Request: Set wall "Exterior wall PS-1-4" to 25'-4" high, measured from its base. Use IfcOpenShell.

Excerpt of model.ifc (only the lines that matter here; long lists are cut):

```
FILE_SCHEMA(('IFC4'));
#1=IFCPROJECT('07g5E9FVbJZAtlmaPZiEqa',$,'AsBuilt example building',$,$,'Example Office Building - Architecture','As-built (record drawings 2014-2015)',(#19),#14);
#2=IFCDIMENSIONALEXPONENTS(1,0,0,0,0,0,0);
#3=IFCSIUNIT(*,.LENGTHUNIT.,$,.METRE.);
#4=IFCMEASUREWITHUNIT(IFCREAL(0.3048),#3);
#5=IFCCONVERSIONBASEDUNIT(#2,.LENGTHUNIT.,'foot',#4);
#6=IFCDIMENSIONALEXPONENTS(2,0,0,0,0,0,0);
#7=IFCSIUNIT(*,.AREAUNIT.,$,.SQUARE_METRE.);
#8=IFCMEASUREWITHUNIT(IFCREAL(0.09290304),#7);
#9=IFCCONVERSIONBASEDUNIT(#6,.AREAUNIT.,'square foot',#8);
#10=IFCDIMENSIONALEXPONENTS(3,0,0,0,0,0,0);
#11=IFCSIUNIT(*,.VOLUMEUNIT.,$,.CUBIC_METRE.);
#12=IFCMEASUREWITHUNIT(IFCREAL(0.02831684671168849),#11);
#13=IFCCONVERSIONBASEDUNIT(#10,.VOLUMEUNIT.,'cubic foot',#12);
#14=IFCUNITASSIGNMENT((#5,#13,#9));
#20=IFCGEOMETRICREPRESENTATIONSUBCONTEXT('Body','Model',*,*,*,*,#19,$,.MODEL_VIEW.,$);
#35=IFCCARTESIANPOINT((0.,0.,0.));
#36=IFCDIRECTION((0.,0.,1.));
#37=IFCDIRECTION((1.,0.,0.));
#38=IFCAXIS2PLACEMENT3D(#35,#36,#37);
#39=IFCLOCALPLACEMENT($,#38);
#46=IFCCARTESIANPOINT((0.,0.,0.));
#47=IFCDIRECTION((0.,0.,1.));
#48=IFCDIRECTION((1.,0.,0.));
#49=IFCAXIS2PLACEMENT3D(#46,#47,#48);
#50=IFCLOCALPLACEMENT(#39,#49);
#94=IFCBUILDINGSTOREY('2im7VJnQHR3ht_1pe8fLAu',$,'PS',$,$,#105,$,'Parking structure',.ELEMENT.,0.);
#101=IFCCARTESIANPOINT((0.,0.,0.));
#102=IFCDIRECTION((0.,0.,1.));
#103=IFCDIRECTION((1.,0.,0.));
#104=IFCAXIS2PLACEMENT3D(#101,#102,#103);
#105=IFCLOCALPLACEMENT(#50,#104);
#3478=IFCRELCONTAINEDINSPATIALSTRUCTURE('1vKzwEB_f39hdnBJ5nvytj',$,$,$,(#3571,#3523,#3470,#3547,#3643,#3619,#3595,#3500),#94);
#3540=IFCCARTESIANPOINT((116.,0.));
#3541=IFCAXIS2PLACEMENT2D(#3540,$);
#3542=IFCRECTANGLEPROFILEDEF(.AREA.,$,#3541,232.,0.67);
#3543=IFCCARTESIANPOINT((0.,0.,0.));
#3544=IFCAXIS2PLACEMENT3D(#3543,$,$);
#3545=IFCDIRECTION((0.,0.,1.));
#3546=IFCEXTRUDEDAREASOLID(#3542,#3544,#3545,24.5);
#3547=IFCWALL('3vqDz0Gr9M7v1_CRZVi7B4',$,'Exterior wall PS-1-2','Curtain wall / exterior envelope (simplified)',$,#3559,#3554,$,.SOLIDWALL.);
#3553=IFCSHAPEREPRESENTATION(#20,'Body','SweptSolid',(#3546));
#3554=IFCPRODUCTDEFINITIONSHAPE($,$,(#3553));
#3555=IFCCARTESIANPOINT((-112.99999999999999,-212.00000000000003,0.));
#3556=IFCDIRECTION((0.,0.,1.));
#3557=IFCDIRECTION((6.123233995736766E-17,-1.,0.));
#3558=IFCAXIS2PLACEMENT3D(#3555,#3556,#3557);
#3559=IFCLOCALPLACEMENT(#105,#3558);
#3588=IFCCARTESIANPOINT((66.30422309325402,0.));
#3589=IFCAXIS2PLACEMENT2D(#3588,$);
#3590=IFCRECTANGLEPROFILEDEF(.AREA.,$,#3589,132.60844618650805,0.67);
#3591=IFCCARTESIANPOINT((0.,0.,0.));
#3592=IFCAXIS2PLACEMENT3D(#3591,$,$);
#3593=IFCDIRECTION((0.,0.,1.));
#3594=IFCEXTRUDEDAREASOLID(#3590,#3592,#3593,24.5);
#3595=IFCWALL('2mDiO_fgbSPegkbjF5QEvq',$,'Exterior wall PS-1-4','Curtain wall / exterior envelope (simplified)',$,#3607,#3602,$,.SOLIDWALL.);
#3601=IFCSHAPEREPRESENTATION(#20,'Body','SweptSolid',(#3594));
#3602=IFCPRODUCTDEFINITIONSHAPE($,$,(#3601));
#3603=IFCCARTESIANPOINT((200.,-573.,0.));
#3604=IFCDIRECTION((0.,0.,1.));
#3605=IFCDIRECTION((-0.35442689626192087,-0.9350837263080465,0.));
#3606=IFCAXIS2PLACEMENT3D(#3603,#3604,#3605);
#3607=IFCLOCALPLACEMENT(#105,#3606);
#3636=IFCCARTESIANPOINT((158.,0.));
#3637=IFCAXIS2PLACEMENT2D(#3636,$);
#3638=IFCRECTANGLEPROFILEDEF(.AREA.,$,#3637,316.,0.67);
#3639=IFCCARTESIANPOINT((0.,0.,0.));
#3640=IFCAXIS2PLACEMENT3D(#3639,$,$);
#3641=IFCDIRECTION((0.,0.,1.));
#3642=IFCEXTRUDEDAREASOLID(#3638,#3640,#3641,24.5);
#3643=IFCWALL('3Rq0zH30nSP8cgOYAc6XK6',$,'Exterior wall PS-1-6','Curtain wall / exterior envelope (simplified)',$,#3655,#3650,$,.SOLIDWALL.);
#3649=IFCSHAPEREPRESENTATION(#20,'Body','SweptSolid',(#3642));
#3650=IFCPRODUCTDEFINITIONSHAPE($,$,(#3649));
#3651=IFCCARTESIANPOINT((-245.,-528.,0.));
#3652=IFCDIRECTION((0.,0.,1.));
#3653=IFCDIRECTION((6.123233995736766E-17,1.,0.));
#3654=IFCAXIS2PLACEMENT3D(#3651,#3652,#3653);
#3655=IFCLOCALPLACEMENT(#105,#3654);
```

```python
import ifcopenshell
import ifcopenshell.geom
import ifcopenshell.util.representation
import ifcopenshell.util.shape
import ifcopenshell.util.unit

model = ifcopenshell.open("model.ifc")
unit_scale = ifcopenshell.util.unit.calculate_unit_scale(model)
settings = ifcopenshell.geom.settings()


def volume(element):
    """Net volume in cubic metres, openings subtracted."""
    shape = ifcopenshell.geom.create_shape(settings, element)
    return ifcopenshell.util.shape.get_volume(shape.geometry)


wall = model.by_guid("2mDiO_fgbSPegkbjF5QEvq")
before = volume(wall)

body = ifcopenshell.util.representation.get_representation(wall, "Model", "Body")
solid = body.Items[0]
old_height = solid.Depth
solid.Depth = 304 * 0.0254 / unit_scale
after = volume(wall)

print(f"height {old_height:g} -> {solid.Depth:g}, volume {before:.3f} -> {after:.3f} m3")

model.write("model_rev.ifc")
```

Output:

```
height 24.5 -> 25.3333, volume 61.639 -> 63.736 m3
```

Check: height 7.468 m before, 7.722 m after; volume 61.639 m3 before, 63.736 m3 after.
